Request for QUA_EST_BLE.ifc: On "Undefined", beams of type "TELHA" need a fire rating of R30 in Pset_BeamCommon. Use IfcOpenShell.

First a look at what the model holds.

```python
import ifcopenshell
import ifcopenshell.util.element

model = ifcopenshell.open("QUA_EST_BLE.ifc")
print(model.schema)
storey = next(s for s in model.by_type("IfcBuildingStorey") if s.Name == "Undefined")
beams = [e for e in ifcopenshell.util.element.get_decomposition(storey) if e.is_a("IfcBeam")]
seen = {}
for e in beams:
    element_type = ifcopenshell.util.element.get_type(e)
    key = (element_type.Name if element_type != e and element_type else None, ifcopenshell.util.element.get_pset(e, "Pset_BeamCommon", "FireRating"))
    seen[key] = seen.get(key, 0) + 1
for (name, value), count in sorted(seen.items(), key=str):
    print(count, "x", name, "|", value)
```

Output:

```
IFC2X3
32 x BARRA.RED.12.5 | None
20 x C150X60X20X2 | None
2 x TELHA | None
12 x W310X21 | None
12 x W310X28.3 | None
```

```python
import ifcopenshell
import ifcopenshell.api.pset
import ifcopenshell.util.element

model = ifcopenshell.open("QUA_EST_BLE.ifc")

storey = next(s for s in model.by_type("IfcBuildingStorey") if s.Name == "Undefined")
beams = [e for e in ifcopenshell.util.element.get_decomposition(storey) if e.is_a("IfcBeam")]

count = 0
for e in beams:
    element_type = ifcopenshell.util.element.get_type(e)
    if element_type in (None, e) or element_type.Name != "TELHA":
        continue
    found = ifcopenshell.util.element.get_pset(e, "Pset_BeamCommon", should_inherit=False)
    if found:
        pset = model.by_id(found["id"])
        if len(ifcopenshell.util.element.get_elements_by_pset(pset)) > 1:
            pset = ifcopenshell.api.pset.unshare_pset(model, products=[e], pset=pset)[0]
    else:
        pset = ifcopenshell.api.pset.add_pset(model, product=e, name="Pset_BeamCommon")
    ifcopenshell.api.pset.edit_pset(model, pset=pset, properties={"FireRating": "R30"})
    count += 1

print(count, "beams updated")

model.write("QUA_EST_BLE_edited.ifc")
```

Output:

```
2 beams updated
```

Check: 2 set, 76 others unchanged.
